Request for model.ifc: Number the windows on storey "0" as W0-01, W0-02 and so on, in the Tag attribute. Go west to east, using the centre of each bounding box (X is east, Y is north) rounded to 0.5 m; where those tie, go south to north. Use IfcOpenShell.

First a look at what the model holds.

```python
import ifcopenshell
import ifcopenshell.util.element
import ifcopenshell.util.placement

model = ifcopenshell.open("model.ifc")
print(model.schema)
storey = next(s for s in model.by_type("IfcBuildingStorey") if s.Name == "0")
windows = [e for e in ifcopenshell.util.element.get_decomposition(storey) if e.is_a("IfcWindow")]
for e in sorted(windows, key=lambda e: e.id()):
    origin = ifcopenshell.util.placement.get_local_placement(e.ObjectPlacement)[:3, 3]
    print(e.id(), e.Tag, e.Name, origin.round(2) + 0.0, sep=" | ")
```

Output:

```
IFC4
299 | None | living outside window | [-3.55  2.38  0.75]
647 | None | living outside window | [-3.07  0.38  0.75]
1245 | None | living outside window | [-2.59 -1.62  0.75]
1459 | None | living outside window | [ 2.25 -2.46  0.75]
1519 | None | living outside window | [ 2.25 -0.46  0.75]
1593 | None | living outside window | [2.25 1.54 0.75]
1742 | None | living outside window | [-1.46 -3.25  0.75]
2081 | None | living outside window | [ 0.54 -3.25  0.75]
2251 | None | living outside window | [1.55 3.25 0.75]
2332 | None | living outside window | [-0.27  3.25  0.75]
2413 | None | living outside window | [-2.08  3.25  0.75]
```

```python
import ifcopenshell
import ifcopenshell.geom
import ifcopenshell.util.element
import ifcopenshell.util.shape

model = ifcopenshell.open("model.ifc")
settings = ifcopenshell.geom.settings()
settings.set("use-world-coords", True)


def centre(element):
    shape = ifcopenshell.geom.create_shape(settings, element)
    return ifcopenshell.util.shape.get_bbox_centroid(shape.geometry)


storey = next(s for s in model.by_type("IfcBuildingStorey") if s.Name == "0")
windows = [e for e in ifcopenshell.util.element.get_decomposition(storey) if e.is_a("IfcWindow")]

# Insertion points can sit at a corner or the storey origin, so sort by the geometry (in metres).
centres = {e: centre(e) for e in windows}
windows.sort(key=lambda e: (round(centres[e][0] / 0.5), centres[e][1]))

for i, e in enumerate(windows, start=1):
    number = f"W0-{i:02d}"
    e.Tag = number
    print(e.id(), number)

model.write("model_rev.ifc")
```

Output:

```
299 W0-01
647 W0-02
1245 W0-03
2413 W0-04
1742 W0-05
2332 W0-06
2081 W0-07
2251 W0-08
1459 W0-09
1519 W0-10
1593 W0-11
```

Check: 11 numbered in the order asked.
